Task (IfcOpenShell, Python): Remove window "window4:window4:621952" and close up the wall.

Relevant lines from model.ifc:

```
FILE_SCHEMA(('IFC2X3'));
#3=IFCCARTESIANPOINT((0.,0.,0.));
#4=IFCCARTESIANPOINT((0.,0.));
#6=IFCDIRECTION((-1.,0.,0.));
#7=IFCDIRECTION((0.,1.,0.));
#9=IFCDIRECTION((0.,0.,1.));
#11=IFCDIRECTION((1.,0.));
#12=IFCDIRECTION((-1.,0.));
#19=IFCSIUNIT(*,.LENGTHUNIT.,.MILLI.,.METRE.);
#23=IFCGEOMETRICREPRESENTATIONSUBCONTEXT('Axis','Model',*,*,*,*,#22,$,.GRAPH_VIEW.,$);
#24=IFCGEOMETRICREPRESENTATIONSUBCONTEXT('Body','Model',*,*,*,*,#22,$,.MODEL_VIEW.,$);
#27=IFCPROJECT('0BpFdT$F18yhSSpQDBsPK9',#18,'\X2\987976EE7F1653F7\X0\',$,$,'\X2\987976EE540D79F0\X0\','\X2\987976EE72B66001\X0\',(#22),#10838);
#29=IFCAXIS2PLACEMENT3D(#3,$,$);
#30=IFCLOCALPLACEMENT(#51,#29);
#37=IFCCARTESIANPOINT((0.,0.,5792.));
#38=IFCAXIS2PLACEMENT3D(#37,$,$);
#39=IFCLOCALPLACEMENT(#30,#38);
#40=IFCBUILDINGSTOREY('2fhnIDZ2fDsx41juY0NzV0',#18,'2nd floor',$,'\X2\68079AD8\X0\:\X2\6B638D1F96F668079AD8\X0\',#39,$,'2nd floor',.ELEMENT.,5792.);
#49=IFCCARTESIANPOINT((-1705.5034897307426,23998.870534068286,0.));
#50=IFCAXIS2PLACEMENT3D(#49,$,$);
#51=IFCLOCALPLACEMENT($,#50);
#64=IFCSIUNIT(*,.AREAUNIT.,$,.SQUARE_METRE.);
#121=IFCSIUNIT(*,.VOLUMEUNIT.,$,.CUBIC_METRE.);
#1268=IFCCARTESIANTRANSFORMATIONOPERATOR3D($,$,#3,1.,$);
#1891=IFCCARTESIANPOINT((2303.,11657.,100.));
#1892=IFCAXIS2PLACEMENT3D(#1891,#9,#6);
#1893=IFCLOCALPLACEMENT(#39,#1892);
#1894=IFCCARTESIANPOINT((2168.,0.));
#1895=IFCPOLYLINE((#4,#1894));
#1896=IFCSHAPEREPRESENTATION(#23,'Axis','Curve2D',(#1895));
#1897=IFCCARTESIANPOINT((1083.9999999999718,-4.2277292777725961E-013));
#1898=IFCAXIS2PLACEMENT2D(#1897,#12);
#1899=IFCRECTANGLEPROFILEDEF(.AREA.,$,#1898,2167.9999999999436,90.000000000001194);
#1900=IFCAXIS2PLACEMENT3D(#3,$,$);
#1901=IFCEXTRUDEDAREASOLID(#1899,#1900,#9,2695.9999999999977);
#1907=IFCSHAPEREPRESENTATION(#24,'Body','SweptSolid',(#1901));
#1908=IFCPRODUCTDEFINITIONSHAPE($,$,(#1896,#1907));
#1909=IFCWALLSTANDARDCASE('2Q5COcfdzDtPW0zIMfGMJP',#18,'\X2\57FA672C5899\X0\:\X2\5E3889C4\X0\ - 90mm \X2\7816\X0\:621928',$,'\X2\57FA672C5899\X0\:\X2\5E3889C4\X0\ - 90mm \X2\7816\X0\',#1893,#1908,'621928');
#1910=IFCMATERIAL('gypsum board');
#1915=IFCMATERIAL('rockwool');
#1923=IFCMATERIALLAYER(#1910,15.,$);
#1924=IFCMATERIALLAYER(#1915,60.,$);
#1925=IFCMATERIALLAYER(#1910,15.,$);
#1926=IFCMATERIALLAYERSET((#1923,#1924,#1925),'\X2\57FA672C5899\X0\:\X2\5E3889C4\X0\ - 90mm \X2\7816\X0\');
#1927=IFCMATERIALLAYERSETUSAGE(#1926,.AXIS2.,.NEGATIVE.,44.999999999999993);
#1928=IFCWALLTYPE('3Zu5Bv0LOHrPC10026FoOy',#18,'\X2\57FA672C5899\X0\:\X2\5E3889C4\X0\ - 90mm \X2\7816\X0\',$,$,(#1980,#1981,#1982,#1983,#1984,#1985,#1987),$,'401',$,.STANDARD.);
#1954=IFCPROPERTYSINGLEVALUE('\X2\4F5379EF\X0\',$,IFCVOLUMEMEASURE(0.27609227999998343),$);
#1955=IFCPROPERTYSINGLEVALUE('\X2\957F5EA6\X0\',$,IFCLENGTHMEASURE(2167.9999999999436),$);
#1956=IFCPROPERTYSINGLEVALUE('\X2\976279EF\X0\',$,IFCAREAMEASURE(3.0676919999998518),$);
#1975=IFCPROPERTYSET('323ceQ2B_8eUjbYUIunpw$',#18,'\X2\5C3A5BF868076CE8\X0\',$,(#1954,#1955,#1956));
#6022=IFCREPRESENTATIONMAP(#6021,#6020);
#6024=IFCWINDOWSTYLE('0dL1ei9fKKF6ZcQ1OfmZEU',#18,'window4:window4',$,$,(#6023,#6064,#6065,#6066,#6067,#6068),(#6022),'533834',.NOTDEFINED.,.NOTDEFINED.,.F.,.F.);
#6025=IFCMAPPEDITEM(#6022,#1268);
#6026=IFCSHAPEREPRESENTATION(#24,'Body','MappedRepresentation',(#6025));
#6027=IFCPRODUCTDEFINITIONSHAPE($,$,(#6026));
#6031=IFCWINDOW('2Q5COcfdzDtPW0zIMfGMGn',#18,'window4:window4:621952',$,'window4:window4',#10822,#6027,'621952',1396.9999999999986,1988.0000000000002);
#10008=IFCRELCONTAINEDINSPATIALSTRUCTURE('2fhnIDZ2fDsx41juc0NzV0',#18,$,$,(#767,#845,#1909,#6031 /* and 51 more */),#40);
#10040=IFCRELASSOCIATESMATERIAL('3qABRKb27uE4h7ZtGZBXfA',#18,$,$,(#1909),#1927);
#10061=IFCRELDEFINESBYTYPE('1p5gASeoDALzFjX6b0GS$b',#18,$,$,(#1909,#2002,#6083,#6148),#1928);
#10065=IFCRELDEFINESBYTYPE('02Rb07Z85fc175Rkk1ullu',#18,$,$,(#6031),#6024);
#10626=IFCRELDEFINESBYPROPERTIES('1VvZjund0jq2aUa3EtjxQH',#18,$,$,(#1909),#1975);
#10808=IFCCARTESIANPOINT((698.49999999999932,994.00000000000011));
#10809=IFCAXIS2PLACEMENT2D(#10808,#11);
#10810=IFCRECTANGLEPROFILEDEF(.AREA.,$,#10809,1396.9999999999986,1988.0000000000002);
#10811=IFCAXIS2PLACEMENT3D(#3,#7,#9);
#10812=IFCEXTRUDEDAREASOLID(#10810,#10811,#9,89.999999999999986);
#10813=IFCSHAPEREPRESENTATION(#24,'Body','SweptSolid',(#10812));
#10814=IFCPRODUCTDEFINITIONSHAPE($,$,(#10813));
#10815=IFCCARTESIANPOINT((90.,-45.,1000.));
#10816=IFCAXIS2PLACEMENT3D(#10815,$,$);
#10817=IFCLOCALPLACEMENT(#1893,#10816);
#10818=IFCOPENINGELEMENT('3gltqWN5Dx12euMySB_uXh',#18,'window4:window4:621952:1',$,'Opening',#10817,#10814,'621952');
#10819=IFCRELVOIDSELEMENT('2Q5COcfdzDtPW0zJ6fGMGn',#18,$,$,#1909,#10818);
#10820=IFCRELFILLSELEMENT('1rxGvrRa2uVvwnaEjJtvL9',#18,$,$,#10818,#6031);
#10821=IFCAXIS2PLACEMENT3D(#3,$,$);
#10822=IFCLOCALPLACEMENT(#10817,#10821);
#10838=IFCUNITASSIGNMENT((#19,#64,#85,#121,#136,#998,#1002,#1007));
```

```python
import ifcopenshell
import ifcopenshell.api.feature
import ifcopenshell.api.pset
import ifcopenshell.api.root
import ifcopenshell.geom
import ifcopenshell.util.element
import ifcopenshell.util.shape
import ifcopenshell.util.unit

model = ifcopenshell.open("model.ifc")
area_scale = ifcopenshell.util.unit.calculate_unit_scale(model, "AREAUNIT")
volume_scale = ifcopenshell.util.unit.calculate_unit_scale(model, "VOLUMEUNIT")
settings = ifcopenshell.geom.settings()


def volume(element):
    """Net volume in cubic metres, openings subtracted."""
    shape = ifcopenshell.geom.create_shape(settings, element)
    return ifcopenshell.util.shape.get_volume(shape.geometry)


window = model.by_guid("2Q5COcfdzDtPW0zIMfGMGn")
opening = window.FillsVoids[0].RelatingOpeningElement
wall = opening.VoidsElements[0].RelatingBuildingElement
before = volume(wall)

ifcopenshell.api.root.remove_product(model, product=window)
ifcopenshell.api.feature.remove_feature(model, feature=opening)

after = volume(wall)
thickness = 0.09  # wall thickness in metres

# Update the wall's stored quantities.
pset = model.by_id(ifcopenshell.util.element.get_pset(wall, "尺寸标注", should_inherit=False)["id"])
ifcopenshell.api.pset.edit_pset(model, pset=pset, properties={
    "体积": model.create_entity("IfcVolumeMeasure", after / volume_scale),
    "面积": model.create_entity("IfcAreaMeasure", after / thickness / area_scale),
})

print(f"wall volume {before:.3f} -> {after:.3f} m3")

model.write("model_v2.ifc")
```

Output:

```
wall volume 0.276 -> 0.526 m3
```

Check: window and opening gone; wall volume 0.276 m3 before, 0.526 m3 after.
